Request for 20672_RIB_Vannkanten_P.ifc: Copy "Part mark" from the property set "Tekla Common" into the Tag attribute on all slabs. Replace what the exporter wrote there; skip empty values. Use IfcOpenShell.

First a look at what the model holds.

```python
import ifcopenshell
import ifcopenshell.util.element

model = ifcopenshell.open("20672_RIB_Vannkanten_P.ifc")
print(model.schema)
slabs = model.by_type("IfcSlab")
print(len(slabs), "slabs")
for e in slabs[:8]:
    source = ifcopenshell.util.element.get_pset(e, "Tekla Common", "Part mark")
    target = e.Tag
    print(e.id(), repr(source), repr(target), sep=" | ")
```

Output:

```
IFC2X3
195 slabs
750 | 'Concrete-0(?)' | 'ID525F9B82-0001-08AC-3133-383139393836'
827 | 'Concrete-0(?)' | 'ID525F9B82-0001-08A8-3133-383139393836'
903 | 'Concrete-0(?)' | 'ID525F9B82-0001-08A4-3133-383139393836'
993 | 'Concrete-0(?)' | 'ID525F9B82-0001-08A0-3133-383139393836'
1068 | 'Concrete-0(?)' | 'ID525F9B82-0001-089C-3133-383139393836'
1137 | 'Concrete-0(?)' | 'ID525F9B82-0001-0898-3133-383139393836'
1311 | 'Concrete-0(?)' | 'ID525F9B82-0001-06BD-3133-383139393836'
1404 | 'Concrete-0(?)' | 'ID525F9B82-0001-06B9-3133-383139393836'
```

```python
import ifcopenshell
import ifcopenshell.util.element

model = ifcopenshell.open("20672_RIB_Vannkanten_P.ifc")

count = 0
for e in model.by_type("IfcSlab"):
    value = ifcopenshell.util.element.get_pset(e, "Tekla Common", "Part mark")
    current = e.Tag
    if not value or not value.strip() or current == value:
        continue
    e.Tag = value
    count += 1

print(count, "slabs updated")

model.write("20672_RIB_Vannkanten_P_v2.ifc")
```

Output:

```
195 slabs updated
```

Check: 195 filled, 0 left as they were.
